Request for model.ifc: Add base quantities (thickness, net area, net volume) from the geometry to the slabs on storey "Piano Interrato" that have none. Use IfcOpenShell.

First a look at what the model holds.

```python
import ifcopenshell
import ifcopenshell.util.element
import ifcopenshell.util.unit

model = ifcopenshell.open("model.ifc")
print(model.schema)
for unit_type in ("LENGTHUNIT", "AREAUNIT", "VOLUMEUNIT"):
    print(unit_type, ifcopenshell.util.unit.calculate_unit_scale(model, unit_type))
storey = next(s for s in model.by_type("IfcBuildingStorey") if s.Name == "Piano Interrato")
slabs = [e for e in ifcopenshell.util.element.get_decomposition(storey) if e.is_a("IfcSlab")]
for e in sorted(slabs, key=lambda e: e.id()):
    print(e.id(), e.is_a(), e.Name, list(ifcopenshell.util.element.get_psets(e, qtos_only=True)), sep=" | ")
```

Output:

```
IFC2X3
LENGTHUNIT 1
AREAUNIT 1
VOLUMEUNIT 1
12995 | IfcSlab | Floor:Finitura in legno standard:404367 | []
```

```python
import ifcopenshell
import ifcopenshell.api.pset
import ifcopenshell.geom
import ifcopenshell.util.element
import ifcopenshell.util.shape
import ifcopenshell.util.unit

model = ifcopenshell.open("model.ifc")
unit_scale = ifcopenshell.util.unit.calculate_unit_scale(model)
area_scale = ifcopenshell.util.unit.calculate_unit_scale(model, "AREAUNIT")
volume_scale = ifcopenshell.util.unit.calculate_unit_scale(model, "VOLUMEUNIT")
settings = ifcopenshell.geom.settings()

storey = next(s for s in model.by_type("IfcBuildingStorey") if s.Name == "Piano Interrato")
slabs = [e for e in ifcopenshell.util.element.get_decomposition(storey) if e.is_a("IfcSlab")]

for e in sorted(slabs, key=lambda e: e.id()):
    if ifcopenshell.util.element.get_psets(e, qtos_only=True, should_inherit=False):
        continue
    # Geometry comes back in metres, in the element's own axes.
    shape = ifcopenshell.geom.create_shape(settings, e)
    values = {
        "Width": ifcopenshell.util.shape.get_z(shape.geometry) / unit_scale,
        "NetArea": ifcopenshell.util.shape.get_footprint_area(shape.geometry) / area_scale,
        "NetVolume": ifcopenshell.util.shape.get_volume(shape.geometry) / volume_scale,
    }
    qto = ifcopenshell.api.pset.add_qto(model, product=e, name="BaseQuantities")
    ifcopenshell.api.pset.edit_qto(model, qto=qto, properties=values)
    print(e.id(), {k: round(v, 3) for k, v in values.items()})

model.write("model_updated.ifc")
```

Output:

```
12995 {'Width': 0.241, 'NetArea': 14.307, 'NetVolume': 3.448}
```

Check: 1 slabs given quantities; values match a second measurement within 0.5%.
